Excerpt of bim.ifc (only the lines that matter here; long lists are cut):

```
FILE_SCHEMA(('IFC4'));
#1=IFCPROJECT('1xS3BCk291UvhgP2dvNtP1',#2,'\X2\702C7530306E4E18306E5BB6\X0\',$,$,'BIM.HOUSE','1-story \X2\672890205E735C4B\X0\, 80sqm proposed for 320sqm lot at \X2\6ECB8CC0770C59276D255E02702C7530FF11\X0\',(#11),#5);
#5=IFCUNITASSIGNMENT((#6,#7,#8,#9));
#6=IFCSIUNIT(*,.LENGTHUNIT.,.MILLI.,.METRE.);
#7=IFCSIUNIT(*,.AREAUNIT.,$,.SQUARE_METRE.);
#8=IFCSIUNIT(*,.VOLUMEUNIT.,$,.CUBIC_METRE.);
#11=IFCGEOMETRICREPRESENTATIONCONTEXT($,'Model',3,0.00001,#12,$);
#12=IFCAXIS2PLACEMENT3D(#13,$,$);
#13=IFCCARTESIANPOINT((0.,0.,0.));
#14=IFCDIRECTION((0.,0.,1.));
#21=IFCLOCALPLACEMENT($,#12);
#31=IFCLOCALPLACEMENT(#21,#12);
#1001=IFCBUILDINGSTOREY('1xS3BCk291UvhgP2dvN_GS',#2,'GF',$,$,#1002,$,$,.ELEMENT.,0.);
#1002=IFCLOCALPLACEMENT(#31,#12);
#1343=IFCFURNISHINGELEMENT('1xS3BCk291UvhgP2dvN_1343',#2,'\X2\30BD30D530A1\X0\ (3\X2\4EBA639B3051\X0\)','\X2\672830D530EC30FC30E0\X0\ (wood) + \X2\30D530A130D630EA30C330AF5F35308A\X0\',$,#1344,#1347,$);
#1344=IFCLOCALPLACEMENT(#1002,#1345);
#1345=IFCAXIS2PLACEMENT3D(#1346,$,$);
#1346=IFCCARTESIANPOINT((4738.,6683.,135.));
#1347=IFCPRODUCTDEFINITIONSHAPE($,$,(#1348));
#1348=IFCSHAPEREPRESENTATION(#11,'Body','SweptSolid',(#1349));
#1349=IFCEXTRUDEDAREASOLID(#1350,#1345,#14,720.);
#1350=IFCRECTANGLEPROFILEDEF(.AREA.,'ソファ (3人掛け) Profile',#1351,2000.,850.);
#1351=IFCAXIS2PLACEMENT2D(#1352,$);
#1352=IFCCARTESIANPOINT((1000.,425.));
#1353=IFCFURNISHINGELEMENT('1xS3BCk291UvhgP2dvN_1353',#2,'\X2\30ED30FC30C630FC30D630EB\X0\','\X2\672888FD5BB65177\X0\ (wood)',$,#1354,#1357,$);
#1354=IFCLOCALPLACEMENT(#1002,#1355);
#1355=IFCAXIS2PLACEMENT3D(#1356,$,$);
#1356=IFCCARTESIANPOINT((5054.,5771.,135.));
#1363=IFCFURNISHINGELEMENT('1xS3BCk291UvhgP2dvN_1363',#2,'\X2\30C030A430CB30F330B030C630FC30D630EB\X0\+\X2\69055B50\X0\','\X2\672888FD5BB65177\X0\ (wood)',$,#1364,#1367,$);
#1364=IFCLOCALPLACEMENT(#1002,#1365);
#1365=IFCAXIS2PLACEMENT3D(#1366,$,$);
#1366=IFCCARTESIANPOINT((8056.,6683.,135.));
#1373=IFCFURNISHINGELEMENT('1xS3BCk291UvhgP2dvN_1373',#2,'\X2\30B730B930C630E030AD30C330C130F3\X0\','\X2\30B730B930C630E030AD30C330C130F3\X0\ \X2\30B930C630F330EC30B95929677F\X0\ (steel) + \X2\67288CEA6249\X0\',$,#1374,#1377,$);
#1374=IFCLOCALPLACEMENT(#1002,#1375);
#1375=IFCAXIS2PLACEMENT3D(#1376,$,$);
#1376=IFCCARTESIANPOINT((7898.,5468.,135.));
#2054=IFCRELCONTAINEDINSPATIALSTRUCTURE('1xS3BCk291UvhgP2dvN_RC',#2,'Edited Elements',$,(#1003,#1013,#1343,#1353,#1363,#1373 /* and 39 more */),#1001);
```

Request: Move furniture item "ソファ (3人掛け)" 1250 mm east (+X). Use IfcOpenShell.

```python
import ifcopenshell
import ifcopenshell.api.geometry
import ifcopenshell.util.placement

model = ifcopenshell.open("bim.ifc")

item = model.by_guid("1xS3BCk291UvhgP2dvN_1343")
matrix = ifcopenshell.util.placement.get_local_placement(item.ObjectPlacement)
matrix[0, 3] += 1250.0
ifcopenshell.api.geometry.edit_object_placement(model, product=item, matrix=matrix, is_si=False)

print(ifcopenshell.util.placement.get_local_placement(item.ObjectPlacement).round(3) + 0.0)

model.write("bim_edited.ifc")
```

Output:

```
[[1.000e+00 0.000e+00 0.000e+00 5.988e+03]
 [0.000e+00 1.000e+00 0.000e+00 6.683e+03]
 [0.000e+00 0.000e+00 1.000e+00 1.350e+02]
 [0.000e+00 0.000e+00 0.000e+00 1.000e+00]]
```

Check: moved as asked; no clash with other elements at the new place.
